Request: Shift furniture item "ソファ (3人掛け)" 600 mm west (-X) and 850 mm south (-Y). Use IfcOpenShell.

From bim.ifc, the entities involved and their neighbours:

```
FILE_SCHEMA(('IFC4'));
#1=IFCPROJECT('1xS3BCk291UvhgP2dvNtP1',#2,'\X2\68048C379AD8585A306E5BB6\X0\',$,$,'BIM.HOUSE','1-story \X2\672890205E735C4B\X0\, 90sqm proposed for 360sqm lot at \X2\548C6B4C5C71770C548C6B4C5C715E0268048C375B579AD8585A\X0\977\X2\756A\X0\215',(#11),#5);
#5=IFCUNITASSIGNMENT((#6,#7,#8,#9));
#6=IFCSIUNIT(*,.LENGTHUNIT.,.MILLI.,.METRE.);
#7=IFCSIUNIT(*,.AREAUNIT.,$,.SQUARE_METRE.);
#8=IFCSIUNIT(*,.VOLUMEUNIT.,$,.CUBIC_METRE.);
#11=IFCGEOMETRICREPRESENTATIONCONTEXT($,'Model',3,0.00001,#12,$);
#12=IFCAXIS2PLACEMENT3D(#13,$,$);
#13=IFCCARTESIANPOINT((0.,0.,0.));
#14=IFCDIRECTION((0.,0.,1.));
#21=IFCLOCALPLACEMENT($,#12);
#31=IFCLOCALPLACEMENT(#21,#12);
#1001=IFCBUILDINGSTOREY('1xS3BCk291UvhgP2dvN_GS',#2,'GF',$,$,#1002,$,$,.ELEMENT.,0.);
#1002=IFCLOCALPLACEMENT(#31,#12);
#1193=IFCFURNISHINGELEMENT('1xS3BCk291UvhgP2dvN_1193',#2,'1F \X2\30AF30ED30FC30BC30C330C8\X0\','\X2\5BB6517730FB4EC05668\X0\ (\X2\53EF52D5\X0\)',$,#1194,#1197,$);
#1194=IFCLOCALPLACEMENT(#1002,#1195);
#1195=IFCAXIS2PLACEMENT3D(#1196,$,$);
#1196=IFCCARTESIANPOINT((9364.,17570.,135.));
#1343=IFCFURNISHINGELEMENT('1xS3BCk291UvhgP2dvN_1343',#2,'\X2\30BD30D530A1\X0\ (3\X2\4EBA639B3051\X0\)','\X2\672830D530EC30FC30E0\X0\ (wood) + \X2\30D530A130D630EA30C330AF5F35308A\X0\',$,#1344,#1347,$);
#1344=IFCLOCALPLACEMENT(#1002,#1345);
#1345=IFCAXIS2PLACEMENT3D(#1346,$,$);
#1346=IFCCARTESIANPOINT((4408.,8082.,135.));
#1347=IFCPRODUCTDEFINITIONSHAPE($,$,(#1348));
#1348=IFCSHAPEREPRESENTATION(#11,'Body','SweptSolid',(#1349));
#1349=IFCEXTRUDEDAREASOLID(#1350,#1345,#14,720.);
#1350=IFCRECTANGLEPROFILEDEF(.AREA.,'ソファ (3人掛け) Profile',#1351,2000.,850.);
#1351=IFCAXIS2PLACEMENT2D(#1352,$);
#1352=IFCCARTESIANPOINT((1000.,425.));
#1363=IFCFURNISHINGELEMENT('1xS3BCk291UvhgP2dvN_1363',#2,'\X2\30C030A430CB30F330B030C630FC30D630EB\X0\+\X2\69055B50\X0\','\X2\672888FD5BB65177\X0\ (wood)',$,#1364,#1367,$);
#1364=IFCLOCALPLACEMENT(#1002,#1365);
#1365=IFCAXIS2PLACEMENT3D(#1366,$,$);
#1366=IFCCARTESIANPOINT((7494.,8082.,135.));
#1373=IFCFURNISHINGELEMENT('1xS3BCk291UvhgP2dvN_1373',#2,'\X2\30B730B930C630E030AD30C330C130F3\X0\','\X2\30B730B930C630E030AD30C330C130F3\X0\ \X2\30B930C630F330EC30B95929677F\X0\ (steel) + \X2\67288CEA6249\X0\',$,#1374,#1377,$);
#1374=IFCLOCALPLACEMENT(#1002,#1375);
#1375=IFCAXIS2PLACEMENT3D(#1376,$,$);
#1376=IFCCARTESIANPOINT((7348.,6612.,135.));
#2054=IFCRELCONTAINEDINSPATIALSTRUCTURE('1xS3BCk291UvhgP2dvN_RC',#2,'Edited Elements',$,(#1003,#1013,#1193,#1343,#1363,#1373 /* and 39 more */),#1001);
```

```python
import ifcopenshell
import ifcopenshell.api.geometry
import ifcopenshell.util.placement
import ifcopenshell.util.unit

model = ifcopenshell.open("bim.ifc")
unit_scale = ifcopenshell.util.unit.calculate_unit_scale(model)

item = model.by_id(1343)
matrix = ifcopenshell.util.placement.get_local_placement(item.ObjectPlacement)
matrix[0, 3] -= 0.6 / unit_scale
matrix[1, 3] -= 0.85 / unit_scale
ifcopenshell.api.geometry.edit_object_placement(model, product=item, matrix=matrix, is_si=False)

print(ifcopenshell.util.placement.get_local_placement(item.ObjectPlacement).round(3) + 0.0)

model.write("bim_rev.ifc")
```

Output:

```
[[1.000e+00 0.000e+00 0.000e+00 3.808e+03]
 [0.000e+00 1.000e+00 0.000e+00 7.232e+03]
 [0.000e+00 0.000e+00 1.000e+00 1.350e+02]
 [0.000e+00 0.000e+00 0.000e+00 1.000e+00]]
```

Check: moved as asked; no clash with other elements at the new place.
